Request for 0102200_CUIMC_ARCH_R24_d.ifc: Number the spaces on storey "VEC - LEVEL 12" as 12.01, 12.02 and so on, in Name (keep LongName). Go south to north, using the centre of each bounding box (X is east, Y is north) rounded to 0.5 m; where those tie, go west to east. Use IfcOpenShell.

First a look at what the model holds.

```python
import ifcopenshell
import ifcopenshell.util.element
import ifcopenshell.util.placement

model = ifcopenshell.open("0102200_CUIMC_ARCH_R24_d.ifc")
print(model.schema)
storey = next(s for s in model.by_type("IfcBuildingStorey") if s.Name == "VEC - LEVEL 12")
spaces = [e for e in ifcopenshell.util.element.get_decomposition(storey) if e.is_a("IfcSpace")]
for e in sorted(spaces, key=lambda e: e.id()):
    origin = ifcopenshell.util.placement.get_local_placement(e.ObjectPlacement)[:3, 3]
    print(e.id(), e.Name, e.LongName, origin.round(2) + 0.0, sep=" | ")
```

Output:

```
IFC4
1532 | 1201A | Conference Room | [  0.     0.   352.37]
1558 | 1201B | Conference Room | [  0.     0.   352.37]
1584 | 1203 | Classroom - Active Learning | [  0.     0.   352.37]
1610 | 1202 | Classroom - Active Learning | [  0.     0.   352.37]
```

```python
import ifcopenshell
import ifcopenshell.geom
import ifcopenshell.util.element
import ifcopenshell.util.shape

model = ifcopenshell.open("0102200_CUIMC_ARCH_R24_d.ifc")
settings = ifcopenshell.geom.settings()
settings.set("use-world-coords", True)


def centre(element):
    shape = ifcopenshell.geom.create_shape(settings, element)
    return ifcopenshell.util.shape.get_bbox_centroid(shape.geometry)


storey = next(s for s in model.by_type("IfcBuildingStorey") if s.Name == "VEC - LEVEL 12")
spaces = [e for e in ifcopenshell.util.element.get_decomposition(storey) if e.is_a("IfcSpace")]

# Insertion points can sit at a corner or the storey origin, so sort by the geometry (in metres).
centres = {e: centre(e) for e in spaces}
spaces.sort(key=lambda e: (round(centres[e][1] / 0.5), centres[e][0]))

for i, e in enumerate(spaces, start=1):
    number = f"12.{i:02d}"
    e.Name = number
    print(e.id(), number)

model.write("0102200_CUIMC_ARCH_R24_d-out.ifc")
```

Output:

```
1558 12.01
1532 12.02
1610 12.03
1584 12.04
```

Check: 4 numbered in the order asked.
